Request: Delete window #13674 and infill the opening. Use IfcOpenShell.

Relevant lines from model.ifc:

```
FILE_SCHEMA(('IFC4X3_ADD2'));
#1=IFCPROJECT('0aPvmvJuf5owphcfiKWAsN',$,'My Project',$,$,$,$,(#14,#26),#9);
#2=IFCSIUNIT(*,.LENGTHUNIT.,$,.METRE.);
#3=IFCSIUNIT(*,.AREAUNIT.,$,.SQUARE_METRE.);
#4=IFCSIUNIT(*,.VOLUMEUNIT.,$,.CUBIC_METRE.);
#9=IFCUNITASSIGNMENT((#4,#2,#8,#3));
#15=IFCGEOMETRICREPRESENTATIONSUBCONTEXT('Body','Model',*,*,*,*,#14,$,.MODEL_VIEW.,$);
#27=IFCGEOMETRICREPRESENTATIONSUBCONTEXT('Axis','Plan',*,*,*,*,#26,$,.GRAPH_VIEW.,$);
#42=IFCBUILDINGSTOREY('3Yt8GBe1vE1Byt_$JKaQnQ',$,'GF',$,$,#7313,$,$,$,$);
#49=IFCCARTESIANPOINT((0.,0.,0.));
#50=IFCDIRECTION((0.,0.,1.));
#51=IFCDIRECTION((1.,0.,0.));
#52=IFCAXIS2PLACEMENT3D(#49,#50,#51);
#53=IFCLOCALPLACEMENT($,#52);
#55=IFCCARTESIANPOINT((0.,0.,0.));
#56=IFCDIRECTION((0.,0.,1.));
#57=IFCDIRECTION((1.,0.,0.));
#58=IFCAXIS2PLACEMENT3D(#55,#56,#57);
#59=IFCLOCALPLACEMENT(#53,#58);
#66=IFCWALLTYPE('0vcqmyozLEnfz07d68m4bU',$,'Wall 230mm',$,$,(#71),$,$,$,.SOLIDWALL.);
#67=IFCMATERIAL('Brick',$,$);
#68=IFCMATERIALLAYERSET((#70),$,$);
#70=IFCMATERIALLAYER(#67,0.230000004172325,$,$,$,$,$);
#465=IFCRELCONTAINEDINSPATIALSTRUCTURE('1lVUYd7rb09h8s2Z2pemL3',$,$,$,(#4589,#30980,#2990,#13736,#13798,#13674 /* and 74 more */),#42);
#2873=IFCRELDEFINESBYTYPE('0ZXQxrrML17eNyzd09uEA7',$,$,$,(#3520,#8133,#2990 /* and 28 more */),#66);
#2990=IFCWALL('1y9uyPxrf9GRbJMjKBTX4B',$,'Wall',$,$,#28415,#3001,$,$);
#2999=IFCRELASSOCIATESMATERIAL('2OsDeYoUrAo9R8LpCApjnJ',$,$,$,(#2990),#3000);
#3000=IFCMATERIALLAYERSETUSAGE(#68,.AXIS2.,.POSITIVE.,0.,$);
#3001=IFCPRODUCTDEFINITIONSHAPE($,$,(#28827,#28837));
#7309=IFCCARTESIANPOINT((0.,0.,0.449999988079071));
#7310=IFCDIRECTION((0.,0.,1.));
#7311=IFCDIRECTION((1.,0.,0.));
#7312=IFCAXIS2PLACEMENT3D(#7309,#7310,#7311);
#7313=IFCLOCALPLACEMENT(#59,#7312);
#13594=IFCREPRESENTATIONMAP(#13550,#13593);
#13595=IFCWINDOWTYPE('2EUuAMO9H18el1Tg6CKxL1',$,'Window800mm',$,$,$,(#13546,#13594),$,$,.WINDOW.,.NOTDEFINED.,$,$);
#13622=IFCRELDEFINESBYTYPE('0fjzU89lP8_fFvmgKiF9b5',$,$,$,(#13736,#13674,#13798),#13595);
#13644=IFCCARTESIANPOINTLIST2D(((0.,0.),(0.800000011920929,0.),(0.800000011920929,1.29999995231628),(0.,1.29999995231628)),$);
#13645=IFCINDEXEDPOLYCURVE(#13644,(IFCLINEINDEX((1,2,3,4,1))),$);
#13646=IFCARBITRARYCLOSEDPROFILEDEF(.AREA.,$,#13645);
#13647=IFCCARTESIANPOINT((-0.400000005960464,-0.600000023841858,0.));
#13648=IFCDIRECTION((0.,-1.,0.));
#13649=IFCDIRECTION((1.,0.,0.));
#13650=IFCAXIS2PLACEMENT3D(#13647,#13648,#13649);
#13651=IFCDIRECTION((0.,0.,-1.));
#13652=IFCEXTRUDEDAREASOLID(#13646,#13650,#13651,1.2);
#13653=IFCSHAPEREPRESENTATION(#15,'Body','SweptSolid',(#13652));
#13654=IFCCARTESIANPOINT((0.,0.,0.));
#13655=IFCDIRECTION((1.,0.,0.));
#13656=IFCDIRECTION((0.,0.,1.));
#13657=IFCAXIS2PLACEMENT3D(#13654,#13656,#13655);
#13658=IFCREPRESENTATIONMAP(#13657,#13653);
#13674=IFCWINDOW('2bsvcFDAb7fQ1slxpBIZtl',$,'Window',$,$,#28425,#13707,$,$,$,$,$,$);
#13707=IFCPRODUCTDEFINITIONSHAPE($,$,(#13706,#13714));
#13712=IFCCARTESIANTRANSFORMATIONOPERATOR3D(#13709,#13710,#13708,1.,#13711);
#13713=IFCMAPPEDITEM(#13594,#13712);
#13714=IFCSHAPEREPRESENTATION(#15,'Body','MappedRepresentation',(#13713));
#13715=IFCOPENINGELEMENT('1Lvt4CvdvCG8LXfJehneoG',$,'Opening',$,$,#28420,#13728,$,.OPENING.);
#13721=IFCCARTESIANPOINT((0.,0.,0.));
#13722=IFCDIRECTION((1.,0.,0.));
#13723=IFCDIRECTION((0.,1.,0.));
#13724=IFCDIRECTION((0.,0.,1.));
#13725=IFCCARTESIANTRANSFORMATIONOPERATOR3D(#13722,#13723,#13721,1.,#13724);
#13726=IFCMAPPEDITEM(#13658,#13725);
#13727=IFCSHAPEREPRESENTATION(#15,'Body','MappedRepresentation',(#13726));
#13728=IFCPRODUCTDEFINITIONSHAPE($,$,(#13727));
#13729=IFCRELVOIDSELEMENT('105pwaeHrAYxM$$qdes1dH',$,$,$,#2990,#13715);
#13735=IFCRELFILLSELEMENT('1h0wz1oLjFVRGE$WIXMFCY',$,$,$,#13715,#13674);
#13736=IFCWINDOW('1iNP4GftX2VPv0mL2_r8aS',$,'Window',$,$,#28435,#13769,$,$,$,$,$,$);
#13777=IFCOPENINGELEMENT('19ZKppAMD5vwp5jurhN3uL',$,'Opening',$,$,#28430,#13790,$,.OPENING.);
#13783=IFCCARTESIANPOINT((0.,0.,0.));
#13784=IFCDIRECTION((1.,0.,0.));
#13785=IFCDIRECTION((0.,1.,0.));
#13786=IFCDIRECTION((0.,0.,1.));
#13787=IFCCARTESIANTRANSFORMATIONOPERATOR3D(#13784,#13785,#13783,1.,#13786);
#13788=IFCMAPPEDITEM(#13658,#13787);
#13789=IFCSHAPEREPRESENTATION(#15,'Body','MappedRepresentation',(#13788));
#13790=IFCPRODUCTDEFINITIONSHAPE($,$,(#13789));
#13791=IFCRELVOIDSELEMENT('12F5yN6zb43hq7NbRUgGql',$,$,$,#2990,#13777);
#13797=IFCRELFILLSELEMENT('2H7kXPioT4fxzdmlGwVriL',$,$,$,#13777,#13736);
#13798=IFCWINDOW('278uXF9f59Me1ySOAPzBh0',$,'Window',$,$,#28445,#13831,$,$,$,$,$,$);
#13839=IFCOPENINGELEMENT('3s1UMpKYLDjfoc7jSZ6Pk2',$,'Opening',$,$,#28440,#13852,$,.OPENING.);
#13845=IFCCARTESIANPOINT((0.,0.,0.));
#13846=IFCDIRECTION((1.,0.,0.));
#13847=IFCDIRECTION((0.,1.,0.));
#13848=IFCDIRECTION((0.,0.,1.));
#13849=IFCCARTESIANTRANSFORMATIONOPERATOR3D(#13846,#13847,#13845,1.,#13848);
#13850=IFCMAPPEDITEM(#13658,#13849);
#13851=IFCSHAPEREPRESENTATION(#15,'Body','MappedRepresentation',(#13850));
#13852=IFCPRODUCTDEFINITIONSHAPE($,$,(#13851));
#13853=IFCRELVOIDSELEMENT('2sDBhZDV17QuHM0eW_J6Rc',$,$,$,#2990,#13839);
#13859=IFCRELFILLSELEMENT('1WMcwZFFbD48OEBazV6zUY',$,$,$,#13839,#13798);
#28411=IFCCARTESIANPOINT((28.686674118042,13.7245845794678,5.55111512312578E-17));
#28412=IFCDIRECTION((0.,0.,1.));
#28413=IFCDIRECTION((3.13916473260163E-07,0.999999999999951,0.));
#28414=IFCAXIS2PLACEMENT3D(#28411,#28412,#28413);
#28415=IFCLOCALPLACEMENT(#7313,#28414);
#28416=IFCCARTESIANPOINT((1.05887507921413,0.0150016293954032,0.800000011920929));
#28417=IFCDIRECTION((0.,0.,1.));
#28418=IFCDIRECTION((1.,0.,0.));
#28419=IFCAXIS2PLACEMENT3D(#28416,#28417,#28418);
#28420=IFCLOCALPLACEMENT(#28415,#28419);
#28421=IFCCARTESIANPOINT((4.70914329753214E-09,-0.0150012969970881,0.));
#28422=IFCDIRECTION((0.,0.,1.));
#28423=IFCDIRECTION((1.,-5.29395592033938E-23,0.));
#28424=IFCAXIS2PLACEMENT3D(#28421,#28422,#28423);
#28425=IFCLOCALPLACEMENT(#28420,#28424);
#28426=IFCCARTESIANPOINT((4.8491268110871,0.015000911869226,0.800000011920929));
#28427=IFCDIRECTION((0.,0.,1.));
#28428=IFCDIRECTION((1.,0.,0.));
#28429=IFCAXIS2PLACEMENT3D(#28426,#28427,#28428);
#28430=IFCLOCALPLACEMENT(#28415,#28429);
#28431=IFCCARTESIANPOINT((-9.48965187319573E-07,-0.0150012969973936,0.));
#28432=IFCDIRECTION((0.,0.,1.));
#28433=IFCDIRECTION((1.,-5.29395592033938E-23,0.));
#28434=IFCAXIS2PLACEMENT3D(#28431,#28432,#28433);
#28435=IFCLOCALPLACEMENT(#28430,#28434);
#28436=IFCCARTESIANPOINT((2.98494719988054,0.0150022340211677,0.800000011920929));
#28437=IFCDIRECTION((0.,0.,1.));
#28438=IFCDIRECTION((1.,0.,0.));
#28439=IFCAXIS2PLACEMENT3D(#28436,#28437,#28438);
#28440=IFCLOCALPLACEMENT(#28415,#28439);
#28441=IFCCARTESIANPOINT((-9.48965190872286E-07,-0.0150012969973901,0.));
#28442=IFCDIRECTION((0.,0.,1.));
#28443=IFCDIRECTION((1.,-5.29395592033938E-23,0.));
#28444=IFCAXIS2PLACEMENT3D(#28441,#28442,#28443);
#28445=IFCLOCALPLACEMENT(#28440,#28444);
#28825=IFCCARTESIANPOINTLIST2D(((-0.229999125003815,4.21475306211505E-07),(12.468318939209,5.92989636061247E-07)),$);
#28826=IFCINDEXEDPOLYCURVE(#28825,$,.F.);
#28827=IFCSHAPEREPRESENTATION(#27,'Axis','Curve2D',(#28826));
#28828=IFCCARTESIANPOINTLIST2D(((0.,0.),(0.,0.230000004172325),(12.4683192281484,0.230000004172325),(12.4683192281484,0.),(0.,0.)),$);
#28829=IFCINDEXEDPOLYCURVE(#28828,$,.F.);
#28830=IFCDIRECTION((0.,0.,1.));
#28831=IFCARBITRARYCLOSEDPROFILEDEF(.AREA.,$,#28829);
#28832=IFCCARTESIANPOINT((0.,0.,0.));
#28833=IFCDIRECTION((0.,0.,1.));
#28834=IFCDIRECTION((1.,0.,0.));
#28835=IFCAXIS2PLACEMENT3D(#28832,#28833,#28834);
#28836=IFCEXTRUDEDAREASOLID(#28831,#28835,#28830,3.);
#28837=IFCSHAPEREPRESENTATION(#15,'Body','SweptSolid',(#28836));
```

```python
import ifcopenshell
import ifcopenshell.api.feature
import ifcopenshell.api.root
import ifcopenshell.geom
import ifcopenshell.util.shape

model = ifcopenshell.open("model.ifc")
settings = ifcopenshell.geom.settings()


def volume(element):
    """Net volume in cubic metres, openings subtracted."""
    shape = ifcopenshell.geom.create_shape(settings, element)
    return ifcopenshell.util.shape.get_volume(shape.geometry)


window = model.by_guid("2bsvcFDAb7fQ1slxpBIZtl")
opening = window.FillsVoids[0].RelatingOpeningElement
wall = opening.VoidsElements[0].RelatingBuildingElement
before = volume(wall)

ifcopenshell.api.root.remove_product(model, product=window)
ifcopenshell.api.feature.remove_feature(model, feature=opening)

after = volume(wall)

print(f"wall volume {before:.3f} -> {after:.3f} m3")

model.write("model_edited.ifc")
```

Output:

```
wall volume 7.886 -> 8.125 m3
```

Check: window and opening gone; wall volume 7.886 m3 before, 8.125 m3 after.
